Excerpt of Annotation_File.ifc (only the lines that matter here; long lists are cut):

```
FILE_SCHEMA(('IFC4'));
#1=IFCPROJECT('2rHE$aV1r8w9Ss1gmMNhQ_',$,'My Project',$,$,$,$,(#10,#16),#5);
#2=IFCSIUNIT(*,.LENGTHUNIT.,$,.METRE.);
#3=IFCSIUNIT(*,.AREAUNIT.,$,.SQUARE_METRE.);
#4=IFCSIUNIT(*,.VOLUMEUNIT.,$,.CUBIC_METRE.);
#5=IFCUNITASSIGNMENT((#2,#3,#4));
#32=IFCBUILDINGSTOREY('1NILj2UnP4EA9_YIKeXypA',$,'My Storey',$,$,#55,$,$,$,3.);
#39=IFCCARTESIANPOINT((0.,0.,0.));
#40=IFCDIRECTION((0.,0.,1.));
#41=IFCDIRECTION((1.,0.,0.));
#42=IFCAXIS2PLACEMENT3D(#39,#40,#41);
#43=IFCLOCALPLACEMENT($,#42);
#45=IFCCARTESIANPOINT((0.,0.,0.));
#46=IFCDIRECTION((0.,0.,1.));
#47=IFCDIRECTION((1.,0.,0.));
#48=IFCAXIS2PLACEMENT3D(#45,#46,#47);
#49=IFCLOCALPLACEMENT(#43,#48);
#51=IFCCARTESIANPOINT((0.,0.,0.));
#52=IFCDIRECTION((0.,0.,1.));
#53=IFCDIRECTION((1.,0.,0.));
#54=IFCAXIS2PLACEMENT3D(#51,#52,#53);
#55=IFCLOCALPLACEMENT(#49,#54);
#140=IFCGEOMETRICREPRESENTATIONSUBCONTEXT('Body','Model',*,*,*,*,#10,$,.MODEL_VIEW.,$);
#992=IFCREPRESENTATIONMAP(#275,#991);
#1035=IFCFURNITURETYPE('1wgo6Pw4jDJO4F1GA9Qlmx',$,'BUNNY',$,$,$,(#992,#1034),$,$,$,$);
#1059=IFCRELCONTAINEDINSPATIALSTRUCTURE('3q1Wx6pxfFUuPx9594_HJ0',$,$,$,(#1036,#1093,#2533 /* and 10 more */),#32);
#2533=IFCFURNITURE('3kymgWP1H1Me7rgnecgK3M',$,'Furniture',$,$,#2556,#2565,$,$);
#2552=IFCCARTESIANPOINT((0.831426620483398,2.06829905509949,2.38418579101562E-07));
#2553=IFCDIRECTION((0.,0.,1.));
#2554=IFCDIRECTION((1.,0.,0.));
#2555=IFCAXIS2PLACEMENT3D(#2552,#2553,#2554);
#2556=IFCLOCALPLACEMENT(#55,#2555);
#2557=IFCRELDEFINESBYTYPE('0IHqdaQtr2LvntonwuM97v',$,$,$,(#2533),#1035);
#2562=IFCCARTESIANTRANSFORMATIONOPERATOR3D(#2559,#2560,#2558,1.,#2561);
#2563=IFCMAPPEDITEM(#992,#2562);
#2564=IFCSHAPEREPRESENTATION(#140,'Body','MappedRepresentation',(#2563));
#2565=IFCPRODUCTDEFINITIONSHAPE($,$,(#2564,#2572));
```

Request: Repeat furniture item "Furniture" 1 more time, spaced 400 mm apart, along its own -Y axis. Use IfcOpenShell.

```python
import ifcopenshell
import ifcopenshell.api.geometry
import ifcopenshell.api.root
import ifcopenshell.util.element
import ifcopenshell.util.placement

model = ifcopenshell.open("Annotation_File.ifc")

source = model.by_id(2533)
base = ifcopenshell.util.placement.get_local_placement(source.ObjectPlacement)
step = -base[:3, 1] * 0.4

for i in range(1, 2):
    copy = ifcopenshell.api.root.copy_class(model, product=source)
    copy.Representation = ifcopenshell.util.element.copy_deep(
        model, source.Representation, exclude=["IfcGeometricRepresentationContext", "IfcRepresentationMap"]
    )
    matrix = base.copy()
    matrix[:3, 3] += i * step
    print("added at", matrix[:3, 3].round(3) + 0.0)
    ifcopenshell.api.geometry.edit_object_placement(model, product=copy, matrix=matrix, is_si=False)

model.write("Annotation_File_rev.ifc")
```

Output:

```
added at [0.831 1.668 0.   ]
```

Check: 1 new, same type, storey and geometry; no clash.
